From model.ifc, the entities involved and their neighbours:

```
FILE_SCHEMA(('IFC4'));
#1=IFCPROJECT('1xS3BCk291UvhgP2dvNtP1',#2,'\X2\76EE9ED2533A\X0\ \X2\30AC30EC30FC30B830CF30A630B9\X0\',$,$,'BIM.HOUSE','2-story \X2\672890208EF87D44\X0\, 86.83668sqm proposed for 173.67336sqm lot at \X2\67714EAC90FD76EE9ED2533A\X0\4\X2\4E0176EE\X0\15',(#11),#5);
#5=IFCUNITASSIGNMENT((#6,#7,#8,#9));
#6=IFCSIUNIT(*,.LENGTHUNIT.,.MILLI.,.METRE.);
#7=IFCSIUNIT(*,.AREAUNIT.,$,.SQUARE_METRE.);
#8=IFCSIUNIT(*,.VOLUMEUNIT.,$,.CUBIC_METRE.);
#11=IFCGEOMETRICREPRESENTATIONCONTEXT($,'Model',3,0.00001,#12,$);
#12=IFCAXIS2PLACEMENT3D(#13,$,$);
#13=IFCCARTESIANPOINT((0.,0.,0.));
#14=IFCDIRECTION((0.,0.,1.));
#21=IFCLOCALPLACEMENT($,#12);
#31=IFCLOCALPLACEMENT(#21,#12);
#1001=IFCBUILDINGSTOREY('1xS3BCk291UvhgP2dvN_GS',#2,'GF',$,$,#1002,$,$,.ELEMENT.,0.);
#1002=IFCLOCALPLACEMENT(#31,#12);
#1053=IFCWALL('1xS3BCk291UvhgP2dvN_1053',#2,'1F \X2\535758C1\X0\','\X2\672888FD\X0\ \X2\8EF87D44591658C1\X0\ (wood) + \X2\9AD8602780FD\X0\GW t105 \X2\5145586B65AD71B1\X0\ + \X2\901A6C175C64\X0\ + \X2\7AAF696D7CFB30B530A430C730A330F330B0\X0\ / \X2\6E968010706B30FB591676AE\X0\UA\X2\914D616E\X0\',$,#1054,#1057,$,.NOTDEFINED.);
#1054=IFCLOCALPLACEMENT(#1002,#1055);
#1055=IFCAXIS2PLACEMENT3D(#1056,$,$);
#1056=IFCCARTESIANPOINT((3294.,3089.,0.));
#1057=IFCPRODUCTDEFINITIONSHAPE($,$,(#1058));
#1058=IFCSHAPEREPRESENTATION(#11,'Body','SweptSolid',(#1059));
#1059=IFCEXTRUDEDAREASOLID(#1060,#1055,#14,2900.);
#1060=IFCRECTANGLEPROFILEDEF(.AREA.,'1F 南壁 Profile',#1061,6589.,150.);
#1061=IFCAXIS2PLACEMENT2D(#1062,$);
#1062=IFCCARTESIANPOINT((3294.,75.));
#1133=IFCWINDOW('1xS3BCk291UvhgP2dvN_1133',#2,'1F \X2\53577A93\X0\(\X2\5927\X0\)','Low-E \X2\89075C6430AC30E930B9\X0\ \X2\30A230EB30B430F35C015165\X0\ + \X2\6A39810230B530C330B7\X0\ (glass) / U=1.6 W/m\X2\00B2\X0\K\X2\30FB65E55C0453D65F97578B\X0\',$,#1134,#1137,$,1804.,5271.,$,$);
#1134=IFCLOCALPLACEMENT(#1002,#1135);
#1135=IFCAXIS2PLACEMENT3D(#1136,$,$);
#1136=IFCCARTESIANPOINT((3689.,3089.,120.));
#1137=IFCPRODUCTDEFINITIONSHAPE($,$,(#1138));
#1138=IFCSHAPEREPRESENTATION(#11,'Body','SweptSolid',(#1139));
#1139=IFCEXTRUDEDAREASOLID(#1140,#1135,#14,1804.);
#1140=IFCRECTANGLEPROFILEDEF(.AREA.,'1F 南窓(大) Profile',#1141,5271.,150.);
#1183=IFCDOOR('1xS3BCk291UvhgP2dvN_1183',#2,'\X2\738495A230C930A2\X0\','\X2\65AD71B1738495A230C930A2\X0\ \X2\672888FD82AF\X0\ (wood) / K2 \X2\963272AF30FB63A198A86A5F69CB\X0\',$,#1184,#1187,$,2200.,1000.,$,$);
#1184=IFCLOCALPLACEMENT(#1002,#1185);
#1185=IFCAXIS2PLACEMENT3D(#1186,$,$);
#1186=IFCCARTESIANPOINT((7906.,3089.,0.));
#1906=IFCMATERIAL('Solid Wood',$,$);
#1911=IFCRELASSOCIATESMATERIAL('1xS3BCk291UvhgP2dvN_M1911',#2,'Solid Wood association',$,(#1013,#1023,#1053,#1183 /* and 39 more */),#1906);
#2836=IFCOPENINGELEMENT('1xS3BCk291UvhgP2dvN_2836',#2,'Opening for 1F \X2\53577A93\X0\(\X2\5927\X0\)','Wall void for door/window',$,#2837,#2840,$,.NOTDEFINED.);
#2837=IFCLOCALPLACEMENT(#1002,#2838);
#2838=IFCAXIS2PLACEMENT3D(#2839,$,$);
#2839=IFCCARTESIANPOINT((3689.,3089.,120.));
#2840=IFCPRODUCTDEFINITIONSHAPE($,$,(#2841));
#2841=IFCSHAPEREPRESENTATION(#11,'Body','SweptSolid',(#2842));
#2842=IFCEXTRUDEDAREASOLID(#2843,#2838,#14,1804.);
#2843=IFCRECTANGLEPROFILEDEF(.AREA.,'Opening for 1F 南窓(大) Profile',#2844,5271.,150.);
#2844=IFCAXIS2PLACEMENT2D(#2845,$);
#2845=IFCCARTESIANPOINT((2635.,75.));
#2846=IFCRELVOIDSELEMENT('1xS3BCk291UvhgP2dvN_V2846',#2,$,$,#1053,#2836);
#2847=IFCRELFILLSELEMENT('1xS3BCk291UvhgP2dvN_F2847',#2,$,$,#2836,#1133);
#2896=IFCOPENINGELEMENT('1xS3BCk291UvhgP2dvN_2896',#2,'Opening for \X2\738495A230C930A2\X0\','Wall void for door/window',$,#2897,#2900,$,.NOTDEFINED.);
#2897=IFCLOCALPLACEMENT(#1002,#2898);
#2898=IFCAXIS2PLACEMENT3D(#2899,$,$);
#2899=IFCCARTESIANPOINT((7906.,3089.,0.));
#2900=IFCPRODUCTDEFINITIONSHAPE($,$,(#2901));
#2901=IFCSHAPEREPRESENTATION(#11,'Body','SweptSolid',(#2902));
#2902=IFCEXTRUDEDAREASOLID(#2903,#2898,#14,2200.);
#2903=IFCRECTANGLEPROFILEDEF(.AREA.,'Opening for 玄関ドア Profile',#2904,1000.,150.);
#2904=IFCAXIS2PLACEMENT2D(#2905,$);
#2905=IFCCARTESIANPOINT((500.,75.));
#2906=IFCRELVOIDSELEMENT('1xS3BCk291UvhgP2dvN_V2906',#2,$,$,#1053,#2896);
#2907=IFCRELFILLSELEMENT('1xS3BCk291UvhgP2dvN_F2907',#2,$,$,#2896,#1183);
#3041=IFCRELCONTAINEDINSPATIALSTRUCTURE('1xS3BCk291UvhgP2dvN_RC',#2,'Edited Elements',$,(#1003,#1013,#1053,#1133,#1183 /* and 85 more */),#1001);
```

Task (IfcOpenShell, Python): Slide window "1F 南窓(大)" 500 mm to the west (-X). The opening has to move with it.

```python
import ifcopenshell
import ifcopenshell.api.geometry
import ifcopenshell.util.placement
import ifcopenshell.util.unit

model = ifcopenshell.open("model.ifc")
unit_scale = ifcopenshell.util.unit.calculate_unit_scale(model)

window = model.by_guid("1xS3BCk291UvhgP2dvN_1133")
opening = window.FillsVoids[0].RelatingOpeningElement
wall = opening.VoidsElements[0].RelatingBuildingElement

wall_matrix = ifcopenshell.util.placement.get_local_placement(wall.ObjectPlacement)
shift = wall_matrix[:3, 0] * -0.5 / unit_scale
before = ifcopenshell.util.placement.get_local_placement(window.ObjectPlacement)[:3, 3].copy()

# The window is not placed relative to its opening, so move both.
for product in (opening, window):
    matrix = ifcopenshell.util.placement.get_local_placement(product.ObjectPlacement)
    matrix[:3, 3] += shift
    ifcopenshell.api.geometry.edit_object_placement(model, product=product, matrix=matrix, is_si=False)

after = ifcopenshell.util.placement.get_local_placement(window.ObjectPlacement)[:3, 3]
print("window moved by", (after - before).round(3) + 0.0)

model.write("model_updated.ifc")
```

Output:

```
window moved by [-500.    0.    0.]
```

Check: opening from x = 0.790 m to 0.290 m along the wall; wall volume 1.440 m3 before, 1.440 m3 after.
